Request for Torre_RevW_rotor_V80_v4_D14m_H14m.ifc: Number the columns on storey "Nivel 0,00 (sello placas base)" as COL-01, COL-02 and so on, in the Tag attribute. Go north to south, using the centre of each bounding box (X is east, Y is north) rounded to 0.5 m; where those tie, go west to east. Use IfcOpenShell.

First a look at what the model holds.

```python
import ifcopenshell
import ifcopenshell.util.element
import ifcopenshell.util.placement

model = ifcopenshell.open("Torre_RevW_rotor_V80_v4_D14m_H14m.ifc")
print(model.schema)
storey = next(s for s in model.by_type("IfcBuildingStorey") if s.Name == "Nivel 0,00 (sello placas base)")
columns = [e for e in ifcopenshell.util.element.get_decomposition(storey) if e.is_a("IfcColumn")]
for e in sorted(columns, key=lambda e: e.id()):
    origin = ifcopenshell.util.placement.get_local_placement(e.ObjectPlacement)[:3, 3]
    print(e.id(), e.Tag, e.Name, origin.round(2) + 0.0, sep=" | ")
```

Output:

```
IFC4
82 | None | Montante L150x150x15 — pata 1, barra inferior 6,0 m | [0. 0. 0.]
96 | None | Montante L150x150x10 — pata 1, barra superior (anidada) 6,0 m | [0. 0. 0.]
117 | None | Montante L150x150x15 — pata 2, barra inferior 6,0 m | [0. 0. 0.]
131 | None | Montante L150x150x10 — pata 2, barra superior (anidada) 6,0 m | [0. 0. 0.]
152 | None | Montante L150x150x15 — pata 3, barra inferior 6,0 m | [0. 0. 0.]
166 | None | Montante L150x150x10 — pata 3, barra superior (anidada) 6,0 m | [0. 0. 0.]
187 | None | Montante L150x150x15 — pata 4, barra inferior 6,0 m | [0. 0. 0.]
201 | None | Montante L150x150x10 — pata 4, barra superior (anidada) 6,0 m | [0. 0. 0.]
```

```python
import ifcopenshell
import ifcopenshell.geom
import ifcopenshell.util.element
import ifcopenshell.util.shape

model = ifcopenshell.open("Torre_RevW_rotor_V80_v4_D14m_H14m.ifc")
settings = ifcopenshell.geom.settings()
settings.set("use-world-coords", True)


def centre(element):
    shape = ifcopenshell.geom.create_shape(settings, element)
    return ifcopenshell.util.shape.get_bbox_centroid(shape.geometry)


storey = next(s for s in model.by_type("IfcBuildingStorey") if s.Name == "Nivel 0,00 (sello placas base)")
columns = [e for e in ifcopenshell.util.element.get_decomposition(storey) if e.is_a("IfcColumn")]

# Insertion points can sit at a corner or the storey origin, so sort by the geometry (in metres).
centres = {e: centre(e) for e in columns}
columns.sort(key=lambda e: (-round(centres[e][1] / 0.5), centres[e][0]))

for i, e in enumerate(columns, start=1):
    number = f"COL-{i:02d}"
    e.Tag = number
    print(e.id(), number)

model.write("Torre_RevW_rotor_V80_v4_D14m_H14m_v2.ifc")
```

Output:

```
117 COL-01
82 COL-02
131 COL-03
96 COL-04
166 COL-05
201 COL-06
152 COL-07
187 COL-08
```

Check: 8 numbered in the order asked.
